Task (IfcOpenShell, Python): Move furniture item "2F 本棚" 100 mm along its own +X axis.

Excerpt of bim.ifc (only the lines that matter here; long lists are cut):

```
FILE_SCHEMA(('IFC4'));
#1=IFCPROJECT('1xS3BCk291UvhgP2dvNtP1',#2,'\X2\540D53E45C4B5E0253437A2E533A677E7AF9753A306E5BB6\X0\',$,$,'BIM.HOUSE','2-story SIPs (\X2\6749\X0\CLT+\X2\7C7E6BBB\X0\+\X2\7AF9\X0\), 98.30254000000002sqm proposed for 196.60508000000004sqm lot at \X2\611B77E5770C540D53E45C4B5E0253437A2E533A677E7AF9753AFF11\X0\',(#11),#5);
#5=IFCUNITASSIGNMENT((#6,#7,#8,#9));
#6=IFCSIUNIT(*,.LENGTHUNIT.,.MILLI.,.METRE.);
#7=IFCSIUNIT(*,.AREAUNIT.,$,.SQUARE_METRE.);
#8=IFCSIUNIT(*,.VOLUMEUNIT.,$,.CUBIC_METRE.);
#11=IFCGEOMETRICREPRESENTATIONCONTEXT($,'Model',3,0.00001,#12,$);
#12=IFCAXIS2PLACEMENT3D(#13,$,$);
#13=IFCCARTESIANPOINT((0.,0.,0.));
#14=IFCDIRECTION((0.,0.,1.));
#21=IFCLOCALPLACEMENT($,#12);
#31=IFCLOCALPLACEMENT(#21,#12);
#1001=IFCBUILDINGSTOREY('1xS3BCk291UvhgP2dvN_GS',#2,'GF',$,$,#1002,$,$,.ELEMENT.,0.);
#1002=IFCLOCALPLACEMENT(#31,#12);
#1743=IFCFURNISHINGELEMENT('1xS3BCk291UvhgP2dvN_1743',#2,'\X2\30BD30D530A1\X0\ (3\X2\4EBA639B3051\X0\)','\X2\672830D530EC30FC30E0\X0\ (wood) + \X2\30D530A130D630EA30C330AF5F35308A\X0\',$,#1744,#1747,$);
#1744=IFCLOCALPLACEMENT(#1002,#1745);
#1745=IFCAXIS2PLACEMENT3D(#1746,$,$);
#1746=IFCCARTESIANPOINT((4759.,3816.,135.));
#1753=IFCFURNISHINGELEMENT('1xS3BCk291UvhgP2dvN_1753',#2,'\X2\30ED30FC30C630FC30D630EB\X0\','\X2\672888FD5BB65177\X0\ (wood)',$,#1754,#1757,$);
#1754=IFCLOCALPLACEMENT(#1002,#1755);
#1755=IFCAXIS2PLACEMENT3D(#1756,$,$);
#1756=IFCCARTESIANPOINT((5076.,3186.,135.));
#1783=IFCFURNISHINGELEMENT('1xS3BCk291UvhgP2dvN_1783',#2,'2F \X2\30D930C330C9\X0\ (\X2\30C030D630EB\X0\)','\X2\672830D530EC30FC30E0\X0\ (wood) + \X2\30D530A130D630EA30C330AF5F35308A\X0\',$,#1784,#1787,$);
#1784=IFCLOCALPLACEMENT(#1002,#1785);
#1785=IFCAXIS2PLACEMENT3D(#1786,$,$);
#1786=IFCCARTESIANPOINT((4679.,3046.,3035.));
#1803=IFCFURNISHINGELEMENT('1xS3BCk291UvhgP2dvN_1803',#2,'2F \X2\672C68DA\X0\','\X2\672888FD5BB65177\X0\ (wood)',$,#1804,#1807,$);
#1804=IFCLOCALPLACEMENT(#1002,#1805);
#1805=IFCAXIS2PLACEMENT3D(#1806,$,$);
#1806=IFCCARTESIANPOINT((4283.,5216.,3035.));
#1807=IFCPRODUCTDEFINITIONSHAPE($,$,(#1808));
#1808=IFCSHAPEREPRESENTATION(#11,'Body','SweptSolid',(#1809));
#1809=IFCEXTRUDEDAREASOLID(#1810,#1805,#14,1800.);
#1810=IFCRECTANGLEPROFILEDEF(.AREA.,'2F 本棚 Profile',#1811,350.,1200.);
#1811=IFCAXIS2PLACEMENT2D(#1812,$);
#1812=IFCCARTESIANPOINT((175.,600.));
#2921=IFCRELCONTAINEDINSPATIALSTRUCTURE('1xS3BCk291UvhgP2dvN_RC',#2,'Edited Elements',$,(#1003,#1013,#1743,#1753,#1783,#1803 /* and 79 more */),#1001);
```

```python
import ifcopenshell
import ifcopenshell.api.geometry
import ifcopenshell.util.placement
import ifcopenshell.util.unit

model = ifcopenshell.open("bim.ifc")
unit_scale = ifcopenshell.util.unit.calculate_unit_scale(model)

item = model.by_id(1803)
matrix = ifcopenshell.util.placement.get_local_placement(item.ObjectPlacement)
matrix[:3, 3] += matrix[:3, 0] * 0.1 / unit_scale
ifcopenshell.api.geometry.edit_object_placement(model, product=item, matrix=matrix, is_si=False)

print(ifcopenshell.util.placement.get_local_placement(item.ObjectPlacement).round(3) + 0.0)

model.write("bim_updated.ifc")
```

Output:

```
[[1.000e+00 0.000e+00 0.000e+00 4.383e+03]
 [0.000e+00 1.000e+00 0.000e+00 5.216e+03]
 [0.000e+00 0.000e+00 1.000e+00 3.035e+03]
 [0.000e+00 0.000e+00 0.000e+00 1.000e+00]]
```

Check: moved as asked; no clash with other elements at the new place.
